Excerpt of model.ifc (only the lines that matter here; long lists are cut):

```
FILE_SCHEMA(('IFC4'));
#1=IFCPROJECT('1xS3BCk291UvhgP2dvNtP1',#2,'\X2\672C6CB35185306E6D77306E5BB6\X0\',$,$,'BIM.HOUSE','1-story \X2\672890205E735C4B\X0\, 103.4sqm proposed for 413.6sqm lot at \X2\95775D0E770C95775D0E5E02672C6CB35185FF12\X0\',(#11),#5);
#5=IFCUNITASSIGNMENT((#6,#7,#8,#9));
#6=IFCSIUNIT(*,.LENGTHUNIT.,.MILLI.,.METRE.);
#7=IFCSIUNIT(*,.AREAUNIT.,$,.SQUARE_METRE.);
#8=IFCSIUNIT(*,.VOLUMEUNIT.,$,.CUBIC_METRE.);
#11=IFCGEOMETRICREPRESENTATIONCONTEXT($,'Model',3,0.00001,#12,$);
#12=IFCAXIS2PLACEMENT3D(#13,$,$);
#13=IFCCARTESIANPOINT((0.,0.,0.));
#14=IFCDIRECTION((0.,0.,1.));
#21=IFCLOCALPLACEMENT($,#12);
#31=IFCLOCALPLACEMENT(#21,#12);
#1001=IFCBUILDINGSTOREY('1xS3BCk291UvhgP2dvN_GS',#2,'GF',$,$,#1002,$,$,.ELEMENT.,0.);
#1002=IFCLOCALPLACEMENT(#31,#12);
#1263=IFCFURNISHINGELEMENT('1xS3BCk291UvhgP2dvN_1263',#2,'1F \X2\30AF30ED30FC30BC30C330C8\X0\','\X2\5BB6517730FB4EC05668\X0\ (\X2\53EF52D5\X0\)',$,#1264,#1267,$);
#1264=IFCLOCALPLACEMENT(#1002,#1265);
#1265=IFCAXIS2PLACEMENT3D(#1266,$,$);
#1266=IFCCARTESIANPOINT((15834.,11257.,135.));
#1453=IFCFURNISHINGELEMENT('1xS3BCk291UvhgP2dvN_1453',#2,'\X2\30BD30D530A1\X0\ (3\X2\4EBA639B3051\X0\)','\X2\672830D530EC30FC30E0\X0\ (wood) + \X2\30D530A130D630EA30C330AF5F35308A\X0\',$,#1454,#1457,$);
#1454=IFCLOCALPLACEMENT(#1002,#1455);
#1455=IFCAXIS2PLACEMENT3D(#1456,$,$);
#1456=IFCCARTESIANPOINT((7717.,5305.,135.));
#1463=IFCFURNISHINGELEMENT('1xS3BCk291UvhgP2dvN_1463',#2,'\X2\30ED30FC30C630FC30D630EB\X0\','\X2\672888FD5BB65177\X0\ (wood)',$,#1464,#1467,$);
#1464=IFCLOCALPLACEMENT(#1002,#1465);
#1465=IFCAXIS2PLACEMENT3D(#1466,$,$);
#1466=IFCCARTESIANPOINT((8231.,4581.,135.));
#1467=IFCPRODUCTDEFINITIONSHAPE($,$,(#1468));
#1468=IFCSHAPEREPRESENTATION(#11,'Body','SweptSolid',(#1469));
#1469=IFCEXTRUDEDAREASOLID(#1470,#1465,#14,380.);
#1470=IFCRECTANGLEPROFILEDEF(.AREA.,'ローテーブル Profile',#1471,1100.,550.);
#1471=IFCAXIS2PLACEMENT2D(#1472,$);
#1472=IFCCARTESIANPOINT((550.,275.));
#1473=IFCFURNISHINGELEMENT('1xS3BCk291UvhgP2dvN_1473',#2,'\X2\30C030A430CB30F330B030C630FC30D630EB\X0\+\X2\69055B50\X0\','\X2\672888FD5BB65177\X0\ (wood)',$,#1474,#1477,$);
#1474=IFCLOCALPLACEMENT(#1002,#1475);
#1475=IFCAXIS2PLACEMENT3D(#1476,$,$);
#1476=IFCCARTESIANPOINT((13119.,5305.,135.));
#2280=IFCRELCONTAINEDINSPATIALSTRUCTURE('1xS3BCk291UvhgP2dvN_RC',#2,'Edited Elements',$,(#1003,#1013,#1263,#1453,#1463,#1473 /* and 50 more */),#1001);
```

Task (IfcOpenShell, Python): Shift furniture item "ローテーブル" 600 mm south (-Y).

```python
import ifcopenshell
import ifcopenshell.api.geometry
import ifcopenshell.util.placement
import ifcopenshell.util.unit

model = ifcopenshell.open("model.ifc")
unit_scale = ifcopenshell.util.unit.calculate_unit_scale(model)

item = model.by_guid("1xS3BCk291UvhgP2dvN_1463")
matrix = ifcopenshell.util.placement.get_local_placement(item.ObjectPlacement)
matrix[1, 3] -= 0.6 / unit_scale
ifcopenshell.api.geometry.edit_object_placement(model, product=item, matrix=matrix, is_si=False)

print(ifcopenshell.util.placement.get_local_placement(item.ObjectPlacement).round(3) + 0.0)

model.write("model_v2.ifc")
```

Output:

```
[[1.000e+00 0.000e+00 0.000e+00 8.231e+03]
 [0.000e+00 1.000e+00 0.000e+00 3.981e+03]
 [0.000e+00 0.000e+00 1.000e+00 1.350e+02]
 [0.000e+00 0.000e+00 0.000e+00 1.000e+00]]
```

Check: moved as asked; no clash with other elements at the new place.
